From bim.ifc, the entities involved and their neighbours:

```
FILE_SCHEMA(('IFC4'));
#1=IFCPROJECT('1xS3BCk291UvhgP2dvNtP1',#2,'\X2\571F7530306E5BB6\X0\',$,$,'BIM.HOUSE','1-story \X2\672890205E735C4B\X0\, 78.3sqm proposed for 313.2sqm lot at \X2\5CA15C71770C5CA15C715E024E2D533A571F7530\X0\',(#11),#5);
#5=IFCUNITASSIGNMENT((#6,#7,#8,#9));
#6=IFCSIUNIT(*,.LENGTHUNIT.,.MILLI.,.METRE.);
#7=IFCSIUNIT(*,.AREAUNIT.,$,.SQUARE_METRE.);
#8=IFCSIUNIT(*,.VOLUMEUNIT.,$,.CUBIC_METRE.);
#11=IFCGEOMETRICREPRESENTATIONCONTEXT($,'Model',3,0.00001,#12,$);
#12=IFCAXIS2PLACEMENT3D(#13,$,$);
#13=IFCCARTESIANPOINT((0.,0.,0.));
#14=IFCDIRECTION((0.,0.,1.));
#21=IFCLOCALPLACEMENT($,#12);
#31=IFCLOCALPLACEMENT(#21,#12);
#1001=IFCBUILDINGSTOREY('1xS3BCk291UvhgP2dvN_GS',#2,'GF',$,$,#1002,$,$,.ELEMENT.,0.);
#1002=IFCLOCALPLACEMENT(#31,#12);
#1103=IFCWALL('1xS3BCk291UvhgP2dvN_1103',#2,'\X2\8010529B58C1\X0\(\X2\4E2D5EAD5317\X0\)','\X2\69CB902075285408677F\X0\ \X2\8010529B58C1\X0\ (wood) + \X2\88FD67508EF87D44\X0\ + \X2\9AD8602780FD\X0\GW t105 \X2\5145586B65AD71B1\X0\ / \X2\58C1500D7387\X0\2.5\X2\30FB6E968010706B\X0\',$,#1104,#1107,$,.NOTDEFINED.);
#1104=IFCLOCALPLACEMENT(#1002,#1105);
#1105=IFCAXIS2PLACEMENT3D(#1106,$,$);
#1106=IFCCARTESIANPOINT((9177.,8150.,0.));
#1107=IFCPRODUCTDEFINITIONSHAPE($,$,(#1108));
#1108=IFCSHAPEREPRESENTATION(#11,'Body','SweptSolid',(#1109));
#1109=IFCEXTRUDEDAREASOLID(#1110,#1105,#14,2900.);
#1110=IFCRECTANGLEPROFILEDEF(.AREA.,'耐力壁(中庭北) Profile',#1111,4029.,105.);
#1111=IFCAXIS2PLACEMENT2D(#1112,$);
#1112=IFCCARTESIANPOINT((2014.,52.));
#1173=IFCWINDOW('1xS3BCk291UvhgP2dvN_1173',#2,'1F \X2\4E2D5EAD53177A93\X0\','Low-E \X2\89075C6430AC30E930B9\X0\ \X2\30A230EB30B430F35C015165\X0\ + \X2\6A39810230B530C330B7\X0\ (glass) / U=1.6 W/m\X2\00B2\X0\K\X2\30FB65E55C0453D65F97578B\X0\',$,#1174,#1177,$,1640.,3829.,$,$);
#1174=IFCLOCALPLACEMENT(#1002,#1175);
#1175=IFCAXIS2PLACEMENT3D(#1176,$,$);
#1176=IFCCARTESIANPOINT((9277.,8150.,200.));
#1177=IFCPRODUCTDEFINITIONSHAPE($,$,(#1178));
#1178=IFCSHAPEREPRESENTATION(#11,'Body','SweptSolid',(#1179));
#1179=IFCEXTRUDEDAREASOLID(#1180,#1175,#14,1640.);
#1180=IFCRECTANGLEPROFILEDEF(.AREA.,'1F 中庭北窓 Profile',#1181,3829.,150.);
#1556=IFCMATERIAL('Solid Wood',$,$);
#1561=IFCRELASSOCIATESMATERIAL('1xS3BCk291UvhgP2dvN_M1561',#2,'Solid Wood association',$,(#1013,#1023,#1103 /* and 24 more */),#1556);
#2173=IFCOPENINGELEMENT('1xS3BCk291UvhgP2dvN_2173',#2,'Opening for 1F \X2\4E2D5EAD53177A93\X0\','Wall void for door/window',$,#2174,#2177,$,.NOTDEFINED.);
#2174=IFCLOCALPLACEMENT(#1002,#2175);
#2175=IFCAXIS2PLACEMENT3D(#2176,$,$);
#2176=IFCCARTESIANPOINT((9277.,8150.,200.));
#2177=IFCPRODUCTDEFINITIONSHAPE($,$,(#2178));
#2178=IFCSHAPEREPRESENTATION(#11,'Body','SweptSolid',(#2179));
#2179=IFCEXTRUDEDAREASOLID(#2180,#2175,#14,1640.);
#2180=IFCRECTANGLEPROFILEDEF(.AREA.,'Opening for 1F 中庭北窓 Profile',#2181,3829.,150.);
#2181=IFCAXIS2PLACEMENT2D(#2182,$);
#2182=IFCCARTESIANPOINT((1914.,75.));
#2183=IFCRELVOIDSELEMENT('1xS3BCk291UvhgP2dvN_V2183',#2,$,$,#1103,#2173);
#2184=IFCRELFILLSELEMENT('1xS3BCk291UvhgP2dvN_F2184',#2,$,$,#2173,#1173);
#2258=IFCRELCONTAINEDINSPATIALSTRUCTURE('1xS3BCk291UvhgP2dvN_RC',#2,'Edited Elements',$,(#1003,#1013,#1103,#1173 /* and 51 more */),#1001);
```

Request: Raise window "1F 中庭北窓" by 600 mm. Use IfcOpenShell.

```python
import numpy as np
import ifcopenshell
import ifcopenshell.api.geometry
import ifcopenshell.util.placement
import ifcopenshell.util.unit

model = ifcopenshell.open("bim.ifc")
unit_scale = ifcopenshell.util.unit.calculate_unit_scale(model)

window = model.by_guid("1xS3BCk291UvhgP2dvN_1173")
opening = window.FillsVoids[0].RelatingOpeningElement
dz = 600.0

shift = np.array([0.0, 0.0, dz])
# The window is not placed relative to its opening, so move both.
for product in (opening, window):
    matrix = ifcopenshell.util.placement.get_local_placement(product.ObjectPlacement)
    matrix[:3, 3] += shift
    ifcopenshell.api.geometry.edit_object_placement(model, product=product, matrix=matrix, is_si=False)

print(f"moved by {dz * unit_scale:+.3f} m")

model.write("bim_updated.ifc")
```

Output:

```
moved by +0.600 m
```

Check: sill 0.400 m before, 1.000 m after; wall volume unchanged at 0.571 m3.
